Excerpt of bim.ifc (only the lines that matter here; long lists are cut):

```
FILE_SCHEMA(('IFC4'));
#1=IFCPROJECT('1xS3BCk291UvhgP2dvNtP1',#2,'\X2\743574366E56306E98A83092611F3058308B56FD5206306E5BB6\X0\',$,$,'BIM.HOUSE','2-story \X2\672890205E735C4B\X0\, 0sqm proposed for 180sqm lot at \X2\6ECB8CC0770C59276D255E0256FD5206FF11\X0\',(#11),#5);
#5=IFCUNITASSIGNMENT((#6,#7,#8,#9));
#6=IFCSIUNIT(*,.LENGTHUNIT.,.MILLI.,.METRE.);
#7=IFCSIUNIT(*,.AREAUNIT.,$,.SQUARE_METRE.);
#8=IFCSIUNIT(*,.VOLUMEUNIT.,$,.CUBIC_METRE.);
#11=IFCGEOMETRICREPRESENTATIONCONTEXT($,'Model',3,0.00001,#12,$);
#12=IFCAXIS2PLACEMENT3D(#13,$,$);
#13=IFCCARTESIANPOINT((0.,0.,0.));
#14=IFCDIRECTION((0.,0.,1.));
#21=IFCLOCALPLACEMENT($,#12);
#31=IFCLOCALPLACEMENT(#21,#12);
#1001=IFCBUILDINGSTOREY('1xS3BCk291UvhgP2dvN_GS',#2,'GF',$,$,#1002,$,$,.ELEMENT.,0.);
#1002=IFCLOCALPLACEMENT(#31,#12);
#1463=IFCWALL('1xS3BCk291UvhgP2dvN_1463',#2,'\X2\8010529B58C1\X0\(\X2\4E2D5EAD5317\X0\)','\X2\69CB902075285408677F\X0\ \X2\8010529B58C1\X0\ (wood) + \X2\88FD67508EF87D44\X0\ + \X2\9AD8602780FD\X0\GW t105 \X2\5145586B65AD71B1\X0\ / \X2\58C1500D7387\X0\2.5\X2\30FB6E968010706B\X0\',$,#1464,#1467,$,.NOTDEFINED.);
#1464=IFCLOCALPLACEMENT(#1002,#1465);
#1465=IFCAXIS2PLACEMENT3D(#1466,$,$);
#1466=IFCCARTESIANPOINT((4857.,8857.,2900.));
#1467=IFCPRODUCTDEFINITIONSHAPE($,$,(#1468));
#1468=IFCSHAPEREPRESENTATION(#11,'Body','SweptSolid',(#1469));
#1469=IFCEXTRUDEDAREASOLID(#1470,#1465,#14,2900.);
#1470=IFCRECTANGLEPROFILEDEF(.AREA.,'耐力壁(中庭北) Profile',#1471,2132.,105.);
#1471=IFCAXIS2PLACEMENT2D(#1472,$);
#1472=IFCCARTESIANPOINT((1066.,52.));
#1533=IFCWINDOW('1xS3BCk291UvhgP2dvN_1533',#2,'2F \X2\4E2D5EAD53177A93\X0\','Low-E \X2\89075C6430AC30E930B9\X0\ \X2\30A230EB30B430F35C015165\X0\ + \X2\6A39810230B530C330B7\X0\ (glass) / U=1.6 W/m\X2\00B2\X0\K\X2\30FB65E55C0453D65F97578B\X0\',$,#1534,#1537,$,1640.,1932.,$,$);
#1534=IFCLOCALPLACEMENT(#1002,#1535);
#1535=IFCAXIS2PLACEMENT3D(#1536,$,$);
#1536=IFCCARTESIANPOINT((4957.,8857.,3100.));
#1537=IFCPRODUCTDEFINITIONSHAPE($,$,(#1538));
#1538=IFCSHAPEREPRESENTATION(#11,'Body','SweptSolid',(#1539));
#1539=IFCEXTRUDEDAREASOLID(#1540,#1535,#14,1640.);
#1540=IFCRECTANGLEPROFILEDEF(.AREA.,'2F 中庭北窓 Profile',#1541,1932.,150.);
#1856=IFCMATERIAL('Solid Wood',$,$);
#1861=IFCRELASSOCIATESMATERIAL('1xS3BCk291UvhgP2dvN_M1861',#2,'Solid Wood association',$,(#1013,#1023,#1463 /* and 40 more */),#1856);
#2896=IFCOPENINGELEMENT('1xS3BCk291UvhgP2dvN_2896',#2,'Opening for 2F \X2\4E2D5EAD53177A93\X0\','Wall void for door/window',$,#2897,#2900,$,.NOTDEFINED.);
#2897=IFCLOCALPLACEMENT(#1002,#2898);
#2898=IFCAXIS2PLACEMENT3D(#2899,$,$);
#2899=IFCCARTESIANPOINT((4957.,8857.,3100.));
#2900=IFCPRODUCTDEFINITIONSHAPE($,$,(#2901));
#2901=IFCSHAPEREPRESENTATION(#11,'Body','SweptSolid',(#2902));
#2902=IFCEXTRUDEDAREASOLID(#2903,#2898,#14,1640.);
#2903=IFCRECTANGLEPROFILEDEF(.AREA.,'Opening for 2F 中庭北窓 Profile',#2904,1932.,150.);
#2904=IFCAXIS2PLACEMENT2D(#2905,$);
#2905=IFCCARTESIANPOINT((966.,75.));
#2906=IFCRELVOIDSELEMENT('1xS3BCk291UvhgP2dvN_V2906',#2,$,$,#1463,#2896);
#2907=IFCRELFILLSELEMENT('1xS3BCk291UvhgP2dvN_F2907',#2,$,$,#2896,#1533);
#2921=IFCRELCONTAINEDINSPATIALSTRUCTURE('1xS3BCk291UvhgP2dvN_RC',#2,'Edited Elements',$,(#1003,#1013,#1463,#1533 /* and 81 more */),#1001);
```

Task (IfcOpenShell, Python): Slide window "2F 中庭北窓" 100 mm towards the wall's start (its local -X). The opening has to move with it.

```python
import ifcopenshell
import ifcopenshell.api.geometry
import ifcopenshell.util.placement
import ifcopenshell.util.unit

model = ifcopenshell.open("bim.ifc")
unit_scale = ifcopenshell.util.unit.calculate_unit_scale(model)

window = model.by_guid("1xS3BCk291UvhgP2dvN_1533")
opening = window.FillsVoids[0].RelatingOpeningElement
wall = opening.VoidsElements[0].RelatingBuildingElement

wall_matrix = ifcopenshell.util.placement.get_local_placement(wall.ObjectPlacement)
shift = wall_matrix[:3, 0] * -0.1 / unit_scale
before = ifcopenshell.util.placement.get_local_placement(window.ObjectPlacement)[:3, 3].copy()

# The window is not placed relative to its opening, so move both.
for product in (opening, window):
    matrix = ifcopenshell.util.placement.get_local_placement(product.ObjectPlacement)
    matrix[:3, 3] += shift
    ifcopenshell.api.geometry.edit_object_placement(model, product=product, matrix=matrix, is_si=False)

after = ifcopenshell.util.placement.get_local_placement(window.ObjectPlacement)[:3, 3]
print("window moved by", (after - before).round(3) + 0.0)

model.write("bim_rev.ifc")
```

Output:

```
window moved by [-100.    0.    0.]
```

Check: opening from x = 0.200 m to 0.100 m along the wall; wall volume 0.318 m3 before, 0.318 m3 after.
